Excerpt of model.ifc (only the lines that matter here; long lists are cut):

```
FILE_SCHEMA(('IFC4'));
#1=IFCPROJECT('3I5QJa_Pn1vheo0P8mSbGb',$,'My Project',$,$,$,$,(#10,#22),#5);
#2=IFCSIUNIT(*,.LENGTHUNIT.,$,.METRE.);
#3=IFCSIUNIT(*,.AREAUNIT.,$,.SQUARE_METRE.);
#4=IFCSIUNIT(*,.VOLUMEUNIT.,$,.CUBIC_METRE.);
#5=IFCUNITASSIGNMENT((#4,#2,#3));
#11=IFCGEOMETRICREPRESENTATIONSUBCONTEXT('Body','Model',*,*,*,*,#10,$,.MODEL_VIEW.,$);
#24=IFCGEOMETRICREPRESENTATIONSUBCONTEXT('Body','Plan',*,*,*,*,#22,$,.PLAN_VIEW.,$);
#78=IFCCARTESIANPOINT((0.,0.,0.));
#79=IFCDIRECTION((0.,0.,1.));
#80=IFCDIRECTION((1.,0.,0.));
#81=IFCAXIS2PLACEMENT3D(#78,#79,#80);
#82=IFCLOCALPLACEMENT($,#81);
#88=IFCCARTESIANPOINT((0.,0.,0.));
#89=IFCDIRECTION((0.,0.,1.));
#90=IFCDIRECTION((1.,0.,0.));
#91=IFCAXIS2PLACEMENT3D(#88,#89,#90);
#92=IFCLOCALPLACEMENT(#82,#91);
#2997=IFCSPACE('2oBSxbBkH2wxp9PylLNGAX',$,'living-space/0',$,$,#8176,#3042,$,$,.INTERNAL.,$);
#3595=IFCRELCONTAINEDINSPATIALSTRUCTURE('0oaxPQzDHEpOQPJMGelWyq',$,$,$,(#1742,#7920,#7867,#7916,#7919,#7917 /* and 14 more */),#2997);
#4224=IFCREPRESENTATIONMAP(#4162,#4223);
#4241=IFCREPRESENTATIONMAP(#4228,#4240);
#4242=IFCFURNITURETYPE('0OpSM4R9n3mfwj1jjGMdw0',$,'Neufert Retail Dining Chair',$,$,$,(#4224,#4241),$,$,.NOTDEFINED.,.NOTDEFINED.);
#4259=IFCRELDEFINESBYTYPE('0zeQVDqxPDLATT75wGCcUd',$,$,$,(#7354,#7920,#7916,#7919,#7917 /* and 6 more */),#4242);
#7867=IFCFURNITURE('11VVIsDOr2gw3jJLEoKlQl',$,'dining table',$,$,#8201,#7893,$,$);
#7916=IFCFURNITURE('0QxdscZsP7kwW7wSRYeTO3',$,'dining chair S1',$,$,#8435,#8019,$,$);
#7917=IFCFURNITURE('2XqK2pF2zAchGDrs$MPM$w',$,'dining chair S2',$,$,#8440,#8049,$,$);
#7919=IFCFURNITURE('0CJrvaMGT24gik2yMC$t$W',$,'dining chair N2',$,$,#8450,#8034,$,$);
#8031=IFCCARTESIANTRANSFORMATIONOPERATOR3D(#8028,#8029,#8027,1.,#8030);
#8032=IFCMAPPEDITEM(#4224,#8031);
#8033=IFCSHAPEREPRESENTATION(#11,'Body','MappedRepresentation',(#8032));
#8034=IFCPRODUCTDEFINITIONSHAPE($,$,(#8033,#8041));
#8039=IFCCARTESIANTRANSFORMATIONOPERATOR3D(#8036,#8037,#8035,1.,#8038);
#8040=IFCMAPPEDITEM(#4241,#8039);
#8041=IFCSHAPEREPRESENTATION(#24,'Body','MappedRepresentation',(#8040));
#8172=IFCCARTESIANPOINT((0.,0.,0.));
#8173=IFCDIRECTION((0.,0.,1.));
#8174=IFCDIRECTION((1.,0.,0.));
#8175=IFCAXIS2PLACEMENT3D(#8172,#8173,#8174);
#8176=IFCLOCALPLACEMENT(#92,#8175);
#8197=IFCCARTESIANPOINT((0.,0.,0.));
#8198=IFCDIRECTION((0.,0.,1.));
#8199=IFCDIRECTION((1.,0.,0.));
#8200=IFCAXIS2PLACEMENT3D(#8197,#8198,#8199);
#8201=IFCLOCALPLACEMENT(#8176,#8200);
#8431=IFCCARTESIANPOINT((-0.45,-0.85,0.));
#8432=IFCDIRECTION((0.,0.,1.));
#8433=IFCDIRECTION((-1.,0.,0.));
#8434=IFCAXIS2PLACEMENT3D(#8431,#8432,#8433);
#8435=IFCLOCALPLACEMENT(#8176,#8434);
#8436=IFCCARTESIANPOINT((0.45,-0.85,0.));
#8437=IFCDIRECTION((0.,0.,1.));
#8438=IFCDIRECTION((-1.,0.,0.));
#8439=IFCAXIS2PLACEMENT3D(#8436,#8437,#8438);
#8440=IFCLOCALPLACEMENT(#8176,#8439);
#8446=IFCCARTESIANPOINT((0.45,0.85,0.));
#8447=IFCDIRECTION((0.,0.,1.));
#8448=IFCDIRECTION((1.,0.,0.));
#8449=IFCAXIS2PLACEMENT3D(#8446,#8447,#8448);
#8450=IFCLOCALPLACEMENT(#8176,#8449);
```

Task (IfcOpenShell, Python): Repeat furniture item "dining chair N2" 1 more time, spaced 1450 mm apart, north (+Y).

```python
import numpy as np
import ifcopenshell
import ifcopenshell.api.geometry
import ifcopenshell.api.root
import ifcopenshell.util.element
import ifcopenshell.util.placement

model = ifcopenshell.open("model.ifc")

source = model.by_guid("0CJrvaMGT24gik2yMC$t$W")
base = ifcopenshell.util.placement.get_local_placement(source.ObjectPlacement)
step = np.array([0.0, 1.0, 0.0]) * 1.45

for i in range(1, 2):
    copy = ifcopenshell.api.root.copy_class(model, product=source)
    copy.Representation = ifcopenshell.util.element.copy_deep(
        model, source.Representation, exclude=["IfcGeometricRepresentationContext", "IfcRepresentationMap"]
    )
    matrix = base.copy()
    matrix[:3, 3] += i * step
    print("added at", matrix[:3, 3].round(3) + 0.0)
    ifcopenshell.api.geometry.edit_object_placement(model, product=copy, matrix=matrix, is_si=False)

model.write("model_v2.ifc")
```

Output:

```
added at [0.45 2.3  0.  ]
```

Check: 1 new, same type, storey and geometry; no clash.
